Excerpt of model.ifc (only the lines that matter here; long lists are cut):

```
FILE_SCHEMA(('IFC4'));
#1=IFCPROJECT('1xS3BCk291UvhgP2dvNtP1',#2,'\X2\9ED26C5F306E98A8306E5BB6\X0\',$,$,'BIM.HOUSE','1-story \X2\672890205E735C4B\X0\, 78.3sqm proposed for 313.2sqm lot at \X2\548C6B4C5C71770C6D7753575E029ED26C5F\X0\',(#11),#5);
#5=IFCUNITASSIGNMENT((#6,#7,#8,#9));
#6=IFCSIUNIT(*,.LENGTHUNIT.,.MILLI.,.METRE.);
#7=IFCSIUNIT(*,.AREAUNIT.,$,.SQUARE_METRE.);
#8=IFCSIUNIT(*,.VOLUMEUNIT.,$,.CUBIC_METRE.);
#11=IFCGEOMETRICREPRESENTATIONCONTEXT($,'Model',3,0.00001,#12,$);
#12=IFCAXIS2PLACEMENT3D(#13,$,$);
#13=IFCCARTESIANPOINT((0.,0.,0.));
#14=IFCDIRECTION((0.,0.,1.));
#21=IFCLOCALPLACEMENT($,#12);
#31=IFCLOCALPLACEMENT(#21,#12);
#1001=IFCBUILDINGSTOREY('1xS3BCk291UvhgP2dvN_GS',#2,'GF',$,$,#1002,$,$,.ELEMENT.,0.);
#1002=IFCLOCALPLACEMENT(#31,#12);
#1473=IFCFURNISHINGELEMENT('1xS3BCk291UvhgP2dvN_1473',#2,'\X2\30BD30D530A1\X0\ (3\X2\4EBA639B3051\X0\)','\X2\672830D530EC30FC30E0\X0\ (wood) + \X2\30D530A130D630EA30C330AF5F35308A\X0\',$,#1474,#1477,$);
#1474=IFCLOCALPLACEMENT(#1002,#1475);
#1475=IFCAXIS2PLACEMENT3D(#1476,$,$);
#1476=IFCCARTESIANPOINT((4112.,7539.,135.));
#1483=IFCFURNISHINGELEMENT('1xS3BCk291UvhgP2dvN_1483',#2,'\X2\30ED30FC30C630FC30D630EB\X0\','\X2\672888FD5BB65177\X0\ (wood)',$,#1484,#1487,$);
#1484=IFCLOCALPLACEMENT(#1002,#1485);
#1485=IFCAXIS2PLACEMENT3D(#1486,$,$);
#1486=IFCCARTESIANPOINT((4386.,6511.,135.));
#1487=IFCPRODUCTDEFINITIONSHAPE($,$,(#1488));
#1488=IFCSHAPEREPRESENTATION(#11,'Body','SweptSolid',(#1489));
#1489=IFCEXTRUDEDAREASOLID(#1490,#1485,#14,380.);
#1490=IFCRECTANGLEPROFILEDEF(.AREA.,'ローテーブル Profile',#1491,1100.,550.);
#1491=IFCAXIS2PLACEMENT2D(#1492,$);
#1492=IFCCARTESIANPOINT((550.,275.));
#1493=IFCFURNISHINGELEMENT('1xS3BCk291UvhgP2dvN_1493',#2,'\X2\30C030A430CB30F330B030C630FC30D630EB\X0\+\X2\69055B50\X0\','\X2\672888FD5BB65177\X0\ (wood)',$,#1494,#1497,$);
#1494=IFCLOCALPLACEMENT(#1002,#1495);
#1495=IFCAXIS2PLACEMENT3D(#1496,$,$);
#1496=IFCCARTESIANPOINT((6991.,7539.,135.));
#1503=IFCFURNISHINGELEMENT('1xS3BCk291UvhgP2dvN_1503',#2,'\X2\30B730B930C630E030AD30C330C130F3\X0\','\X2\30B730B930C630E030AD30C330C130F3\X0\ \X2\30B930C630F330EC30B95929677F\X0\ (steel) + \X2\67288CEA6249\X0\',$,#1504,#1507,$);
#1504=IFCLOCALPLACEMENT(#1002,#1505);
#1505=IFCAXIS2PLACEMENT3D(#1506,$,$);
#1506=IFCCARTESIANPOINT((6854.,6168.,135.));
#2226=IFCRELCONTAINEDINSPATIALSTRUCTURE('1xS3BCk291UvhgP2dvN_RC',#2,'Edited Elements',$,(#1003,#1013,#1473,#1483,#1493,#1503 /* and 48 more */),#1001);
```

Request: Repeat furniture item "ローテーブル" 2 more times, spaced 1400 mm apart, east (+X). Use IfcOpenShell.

```python
import numpy as np
import ifcopenshell
import ifcopenshell.api.geometry
import ifcopenshell.api.root
import ifcopenshell.util.element
import ifcopenshell.util.placement
import ifcopenshell.util.unit

model = ifcopenshell.open("model.ifc")
unit_scale = ifcopenshell.util.unit.calculate_unit_scale(model)


def reuse_history(source, copy):
    """copy_class also copies each property set's owner history, people and application; keep the originals."""
    for rel in copy.IsDefinedBy:
        if rel.is_a("IfcRelDefinesByProperties") and (history := rel.RelatingPropertyDefinition.OwnerHistory):
            rel.RelatingPropertyDefinition.OwnerHistory = source.OwnerHistory
            ifcopenshell.util.element.remove_deep2(model, history)


source = model.by_id(1483)
base = ifcopenshell.util.placement.get_local_placement(source.ObjectPlacement)
step = np.array([1.0, 0.0, 0.0]) * 1.4 / unit_scale

for i in range(1, 3):
    copy = ifcopenshell.api.root.copy_class(model, product=source)
    copy.Representation = ifcopenshell.util.element.copy_deep(
        model, source.Representation, exclude=["IfcGeometricRepresentationContext", "IfcRepresentationMap"]
    )
    reuse_history(source, copy)
    matrix = base.copy()
    matrix[:3, 3] += i * step
    print("added at", matrix[:3, 3].round(3) + 0.0)
    ifcopenshell.api.geometry.edit_object_placement(model, product=copy, matrix=matrix, is_si=False)

model.write("model_rev.ifc")
```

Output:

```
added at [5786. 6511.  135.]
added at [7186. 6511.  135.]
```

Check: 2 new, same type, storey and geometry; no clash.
